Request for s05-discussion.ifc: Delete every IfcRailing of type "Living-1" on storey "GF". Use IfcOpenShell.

First a look at what the model holds.

```python
import ifcopenshell
import ifcopenshell.util.element

model = ifcopenshell.open("s05-discussion.ifc")
print(model.schema)
storey = next(s for s in model.by_type("IfcBuildingStorey") if s.Name == "GF")
railings = [e for e in ifcopenshell.util.element.get_decomposition(storey) if e.is_a("IfcRailing")]
seen = {}
for e in railings:
    element_type = ifcopenshell.util.element.get_type(e)
    name = element_type.Name if element_type not in (None, e) else None
    seen[name] = seen.get(name, 0) + 1
for name, count in sorted(seen.items(), key=str):
    print(count, "x", name)
```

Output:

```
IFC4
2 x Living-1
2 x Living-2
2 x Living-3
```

```python
import ifcopenshell
import ifcopenshell.api.root
import ifcopenshell.util.element

model = ifcopenshell.open("s05-discussion.ifc")

storey = next(s for s in model.by_type("IfcBuildingStorey") if s.Name == "GF")
railings = [e for e in ifcopenshell.util.element.get_decomposition(storey) if e.is_a("IfcRailing")]
targets = [e for e in railings if (t := ifcopenshell.util.element.get_type(e)) not in (None, e) and t.Name == "Living-1"]

for e in targets:
    ifcopenshell.api.root.remove_product(model, product=e)
print(len(targets), "removed")

model.write("s05-discussion_rev.ifc")
```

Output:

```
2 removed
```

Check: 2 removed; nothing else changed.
